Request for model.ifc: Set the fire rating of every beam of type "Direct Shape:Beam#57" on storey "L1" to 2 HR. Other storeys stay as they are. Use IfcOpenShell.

First a look at what the model holds.

```python
import ifcopenshell
import ifcopenshell.util.element

model = ifcopenshell.open("model.ifc")
print(model.schema)
storey = next(s for s in model.by_type("IfcBuildingStorey") if s.Name == "L1")
beams = [e for e in ifcopenshell.util.element.get_decomposition(storey) if e.is_a("IfcBeam")]
seen = {}
for e in beams:
    element_type = ifcopenshell.util.element.get_type(e)
    key = (element_type.Name if element_type != e and element_type else None, ifcopenshell.util.element.get_pset(e, "Pset_BeamCommon", "FireRating"))
    seen[key] = seen.get(key, 0) + 1
for (name, value), count in sorted(seen.items(), key=str):
    print(count, "x", name, "|", value)
```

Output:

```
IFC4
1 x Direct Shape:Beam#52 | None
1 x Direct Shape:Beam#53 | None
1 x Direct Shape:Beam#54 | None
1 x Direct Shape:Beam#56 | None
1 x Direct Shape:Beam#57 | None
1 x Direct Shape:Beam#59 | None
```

```python
import ifcopenshell
import ifcopenshell.api.pset
import ifcopenshell.util.element

model = ifcopenshell.open("model.ifc")

storey = next(s for s in model.by_type("IfcBuildingStorey") if s.Name == "L1")
beams = [e for e in ifcopenshell.util.element.get_decomposition(storey) if e.is_a("IfcBeam")]

count = 0
for e in beams:
    element_type = ifcopenshell.util.element.get_type(e)
    if element_type in (None, e) or element_type.Name != "Direct Shape:Beam#57":
        continue
    # add_pset returns the element's existing set when there is one.
    pset = ifcopenshell.api.pset.add_pset(model, product=e, name="Pset_BeamCommon")
    ifcopenshell.api.pset.edit_pset(model, pset=pset, properties={"FireRating": "2 HR"})
    count += 1

print(count, "beams updated")

model.write("model_updated.ifc")
```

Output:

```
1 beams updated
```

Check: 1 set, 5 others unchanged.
